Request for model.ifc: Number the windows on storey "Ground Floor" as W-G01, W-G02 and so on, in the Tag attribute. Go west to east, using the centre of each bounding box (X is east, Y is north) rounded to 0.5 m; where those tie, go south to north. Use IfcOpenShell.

First a look at what the model holds.

```python
import ifcopenshell
import ifcopenshell.util.element
import ifcopenshell.util.placement

model = ifcopenshell.open("model.ifc")
print(model.schema)
storey = next(s for s in model.by_type("IfcBuildingStorey") if s.Name == "Ground Floor")
windows = [e for e in ifcopenshell.util.element.get_decomposition(storey) if e.is_a("IfcWindow")]
for e in sorted(windows, key=lambda e: e.id()):
    origin = ifcopenshell.util.placement.get_local_placement(e.ObjectPlacement)[:3, 3]
    print(e.id(), e.Tag, e.Name, origin.round(2) + 0.0, sep=" | ")
```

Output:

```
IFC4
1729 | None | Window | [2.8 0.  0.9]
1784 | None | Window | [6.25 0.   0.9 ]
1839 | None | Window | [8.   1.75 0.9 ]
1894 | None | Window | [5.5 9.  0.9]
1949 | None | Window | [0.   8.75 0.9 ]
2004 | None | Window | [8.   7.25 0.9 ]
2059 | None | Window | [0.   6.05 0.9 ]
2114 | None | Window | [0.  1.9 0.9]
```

```python
import ifcopenshell
import ifcopenshell.geom
import ifcopenshell.util.element
import ifcopenshell.util.shape

model = ifcopenshell.open("model.ifc")
settings = ifcopenshell.geom.settings()
settings.set("use-world-coords", True)


def centre(element):
    shape = ifcopenshell.geom.create_shape(settings, element)
    return ifcopenshell.util.shape.get_bbox_centroid(shape.geometry)


storey = next(s for s in model.by_type("IfcBuildingStorey") if s.Name == "Ground Floor")
windows = [e for e in ifcopenshell.util.element.get_decomposition(storey) if e.is_a("IfcWindow")]

# Insertion points can sit at a corner or the storey origin, so sort by the geometry (in metres).
centres = {e: centre(e) for e in windows}
windows.sort(key=lambda e: (round(centres[e][0] / 0.5), centres[e][1]))

for i, e in enumerate(windows, start=1):
    number = f"W-G{i:02d}"
    e.Tag = number
    print(e.id(), number)

model.write("model_updated.ifc")
```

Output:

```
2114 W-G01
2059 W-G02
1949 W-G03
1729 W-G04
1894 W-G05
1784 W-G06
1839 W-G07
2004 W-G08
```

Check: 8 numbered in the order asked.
